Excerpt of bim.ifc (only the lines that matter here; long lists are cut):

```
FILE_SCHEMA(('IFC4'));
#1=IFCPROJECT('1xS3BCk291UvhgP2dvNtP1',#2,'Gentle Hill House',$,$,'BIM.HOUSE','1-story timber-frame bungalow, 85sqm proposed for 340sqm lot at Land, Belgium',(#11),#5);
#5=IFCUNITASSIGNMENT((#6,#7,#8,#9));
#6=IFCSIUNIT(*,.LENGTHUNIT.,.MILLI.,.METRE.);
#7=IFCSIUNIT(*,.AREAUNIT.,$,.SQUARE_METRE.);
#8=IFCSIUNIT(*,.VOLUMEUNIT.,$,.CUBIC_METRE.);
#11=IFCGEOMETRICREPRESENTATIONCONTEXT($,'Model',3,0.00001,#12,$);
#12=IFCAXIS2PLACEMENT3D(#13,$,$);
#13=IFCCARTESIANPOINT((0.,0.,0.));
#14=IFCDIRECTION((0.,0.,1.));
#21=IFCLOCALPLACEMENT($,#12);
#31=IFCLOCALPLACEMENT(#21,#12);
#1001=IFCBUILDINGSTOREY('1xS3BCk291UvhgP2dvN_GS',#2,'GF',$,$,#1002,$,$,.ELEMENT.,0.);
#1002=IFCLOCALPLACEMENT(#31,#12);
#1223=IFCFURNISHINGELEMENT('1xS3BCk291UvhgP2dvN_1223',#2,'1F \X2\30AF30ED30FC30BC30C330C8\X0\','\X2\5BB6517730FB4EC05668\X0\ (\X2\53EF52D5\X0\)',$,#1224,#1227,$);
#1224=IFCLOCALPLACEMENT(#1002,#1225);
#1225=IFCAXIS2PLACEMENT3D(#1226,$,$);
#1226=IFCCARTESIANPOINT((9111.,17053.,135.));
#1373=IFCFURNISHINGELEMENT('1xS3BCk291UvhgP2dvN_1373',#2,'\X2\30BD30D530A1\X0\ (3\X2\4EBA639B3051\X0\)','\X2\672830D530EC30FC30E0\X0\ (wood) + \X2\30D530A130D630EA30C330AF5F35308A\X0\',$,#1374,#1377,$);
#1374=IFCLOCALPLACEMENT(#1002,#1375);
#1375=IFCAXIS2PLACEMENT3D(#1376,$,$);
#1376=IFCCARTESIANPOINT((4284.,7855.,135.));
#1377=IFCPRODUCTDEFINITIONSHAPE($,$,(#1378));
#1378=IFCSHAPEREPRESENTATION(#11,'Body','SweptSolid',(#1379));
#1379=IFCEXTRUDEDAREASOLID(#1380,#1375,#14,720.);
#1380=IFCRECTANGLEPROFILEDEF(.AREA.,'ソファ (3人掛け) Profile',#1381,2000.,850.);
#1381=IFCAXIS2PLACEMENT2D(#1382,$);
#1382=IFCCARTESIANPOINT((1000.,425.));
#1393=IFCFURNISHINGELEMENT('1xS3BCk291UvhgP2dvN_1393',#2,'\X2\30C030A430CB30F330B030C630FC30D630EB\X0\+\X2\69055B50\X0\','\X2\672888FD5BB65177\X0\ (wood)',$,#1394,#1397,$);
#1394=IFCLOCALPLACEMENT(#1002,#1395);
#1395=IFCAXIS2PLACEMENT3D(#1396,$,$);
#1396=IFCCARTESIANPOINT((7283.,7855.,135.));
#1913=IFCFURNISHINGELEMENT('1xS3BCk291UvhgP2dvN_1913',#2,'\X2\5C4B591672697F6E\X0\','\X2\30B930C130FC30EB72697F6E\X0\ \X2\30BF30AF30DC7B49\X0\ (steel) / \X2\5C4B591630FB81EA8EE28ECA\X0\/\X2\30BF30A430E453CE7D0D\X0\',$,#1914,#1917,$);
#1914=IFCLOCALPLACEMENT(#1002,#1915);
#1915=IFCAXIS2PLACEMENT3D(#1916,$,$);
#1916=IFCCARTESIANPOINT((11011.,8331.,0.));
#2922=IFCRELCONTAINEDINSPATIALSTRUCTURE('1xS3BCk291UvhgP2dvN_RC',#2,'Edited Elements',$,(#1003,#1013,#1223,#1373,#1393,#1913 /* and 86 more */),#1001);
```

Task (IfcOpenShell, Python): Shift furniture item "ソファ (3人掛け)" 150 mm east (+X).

```python
import ifcopenshell
import ifcopenshell.api.geometry
import ifcopenshell.util.placement

model = ifcopenshell.open("bim.ifc")

item = model.by_id(1373)
matrix = ifcopenshell.util.placement.get_local_placement(item.ObjectPlacement)
matrix[0, 3] += 150.0
ifcopenshell.api.geometry.edit_object_placement(model, product=item, matrix=matrix, is_si=False)

print(ifcopenshell.util.placement.get_local_placement(item.ObjectPlacement).round(3) + 0.0)

model.write("bim_v2.ifc")
```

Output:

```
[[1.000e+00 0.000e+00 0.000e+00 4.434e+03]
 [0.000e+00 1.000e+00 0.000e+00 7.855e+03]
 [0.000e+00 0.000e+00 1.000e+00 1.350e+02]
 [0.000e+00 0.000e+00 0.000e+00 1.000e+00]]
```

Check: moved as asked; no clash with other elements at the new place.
